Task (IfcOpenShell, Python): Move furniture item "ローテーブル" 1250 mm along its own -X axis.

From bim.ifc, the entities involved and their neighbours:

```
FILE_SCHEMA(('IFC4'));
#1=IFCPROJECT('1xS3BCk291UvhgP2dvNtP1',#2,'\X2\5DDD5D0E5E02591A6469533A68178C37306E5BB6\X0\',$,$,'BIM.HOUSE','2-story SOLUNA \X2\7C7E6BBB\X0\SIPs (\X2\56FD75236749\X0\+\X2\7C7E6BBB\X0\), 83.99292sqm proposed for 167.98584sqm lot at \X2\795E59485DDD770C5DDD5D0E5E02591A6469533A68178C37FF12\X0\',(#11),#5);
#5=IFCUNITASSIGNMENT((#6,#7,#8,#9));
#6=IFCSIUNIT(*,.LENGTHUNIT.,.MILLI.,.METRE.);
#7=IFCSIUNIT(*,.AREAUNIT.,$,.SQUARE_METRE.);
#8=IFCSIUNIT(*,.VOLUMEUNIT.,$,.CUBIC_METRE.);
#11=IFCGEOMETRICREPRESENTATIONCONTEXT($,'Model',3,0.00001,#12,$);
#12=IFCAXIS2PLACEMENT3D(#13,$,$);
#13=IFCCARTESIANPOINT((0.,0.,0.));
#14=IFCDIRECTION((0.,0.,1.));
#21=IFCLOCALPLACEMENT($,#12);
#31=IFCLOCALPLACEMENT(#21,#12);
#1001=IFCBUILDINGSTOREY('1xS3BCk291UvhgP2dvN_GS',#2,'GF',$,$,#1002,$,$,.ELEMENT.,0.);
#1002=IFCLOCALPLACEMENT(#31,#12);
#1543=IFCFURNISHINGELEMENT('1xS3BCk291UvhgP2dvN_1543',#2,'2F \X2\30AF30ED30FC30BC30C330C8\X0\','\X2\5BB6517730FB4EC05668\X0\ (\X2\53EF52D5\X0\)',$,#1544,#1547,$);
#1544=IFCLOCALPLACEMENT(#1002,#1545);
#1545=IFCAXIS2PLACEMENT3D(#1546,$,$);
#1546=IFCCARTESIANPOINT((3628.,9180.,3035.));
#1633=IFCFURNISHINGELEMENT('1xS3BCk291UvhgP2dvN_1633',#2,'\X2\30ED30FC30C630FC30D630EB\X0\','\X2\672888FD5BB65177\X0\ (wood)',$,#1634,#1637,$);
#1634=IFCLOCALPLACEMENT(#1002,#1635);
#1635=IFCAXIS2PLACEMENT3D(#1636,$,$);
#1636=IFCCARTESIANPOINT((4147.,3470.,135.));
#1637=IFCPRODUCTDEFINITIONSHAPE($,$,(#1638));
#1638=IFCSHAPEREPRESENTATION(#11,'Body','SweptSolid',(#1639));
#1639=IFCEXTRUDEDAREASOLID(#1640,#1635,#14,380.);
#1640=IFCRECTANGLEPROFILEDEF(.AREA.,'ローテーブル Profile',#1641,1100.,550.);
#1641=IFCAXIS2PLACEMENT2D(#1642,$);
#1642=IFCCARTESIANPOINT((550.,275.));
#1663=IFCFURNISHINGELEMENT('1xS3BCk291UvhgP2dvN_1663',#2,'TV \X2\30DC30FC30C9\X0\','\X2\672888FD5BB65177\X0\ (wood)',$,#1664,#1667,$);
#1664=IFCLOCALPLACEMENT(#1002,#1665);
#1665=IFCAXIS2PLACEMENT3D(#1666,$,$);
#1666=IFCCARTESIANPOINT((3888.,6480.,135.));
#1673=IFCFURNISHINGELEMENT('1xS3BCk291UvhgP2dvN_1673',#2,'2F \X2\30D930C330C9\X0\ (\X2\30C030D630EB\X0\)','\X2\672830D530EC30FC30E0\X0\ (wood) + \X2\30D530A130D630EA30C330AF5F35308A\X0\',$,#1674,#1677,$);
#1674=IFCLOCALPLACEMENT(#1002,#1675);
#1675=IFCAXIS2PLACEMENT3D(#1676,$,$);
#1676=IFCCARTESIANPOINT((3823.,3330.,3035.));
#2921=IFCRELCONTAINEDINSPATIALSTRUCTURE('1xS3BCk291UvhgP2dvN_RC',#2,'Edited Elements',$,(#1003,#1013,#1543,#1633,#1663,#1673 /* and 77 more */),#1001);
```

```python
import ifcopenshell
import ifcopenshell.api.geometry
import ifcopenshell.util.placement
import ifcopenshell.util.unit

model = ifcopenshell.open("bim.ifc")
unit_scale = ifcopenshell.util.unit.calculate_unit_scale(model)

item = model.by_guid("1xS3BCk291UvhgP2dvN_1633")
matrix = ifcopenshell.util.placement.get_local_placement(item.ObjectPlacement)
matrix[:3, 3] -= matrix[:3, 0] * 1.25 / unit_scale
ifcopenshell.api.geometry.edit_object_placement(model, product=item, matrix=matrix, is_si=False)

print(ifcopenshell.util.placement.get_local_placement(item.ObjectPlacement).round(3) + 0.0)

model.write("bim-out.ifc")
```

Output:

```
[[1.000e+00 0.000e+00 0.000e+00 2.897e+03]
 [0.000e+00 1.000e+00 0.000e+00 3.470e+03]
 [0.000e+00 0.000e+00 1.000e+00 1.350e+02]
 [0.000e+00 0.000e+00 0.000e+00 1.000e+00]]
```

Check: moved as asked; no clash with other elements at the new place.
